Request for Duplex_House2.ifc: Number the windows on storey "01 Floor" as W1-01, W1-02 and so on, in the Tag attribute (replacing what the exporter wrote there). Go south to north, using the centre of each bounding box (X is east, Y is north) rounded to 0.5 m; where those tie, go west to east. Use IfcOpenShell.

First a look at what the model holds.

```python
import ifcopenshell
import ifcopenshell.util.element
import ifcopenshell.util.placement

model = ifcopenshell.open("Duplex_House2.ifc")
print(model.schema)
storey = next(s for s in model.by_type("IfcBuildingStorey") if s.Name == "01 Floor")
windows = [e for e in ifcopenshell.util.element.get_decomposition(storey) if e.is_a("IfcWindow")]
for e in sorted(windows, key=lambda e: e.id()):
    origin = ifcopenshell.util.placement.get_local_placement(e.ObjectPlacement)[:3, 3]
    print(e.id(), e.Tag, e.Name, origin.round(2) + 0.0, sep=" | ")
```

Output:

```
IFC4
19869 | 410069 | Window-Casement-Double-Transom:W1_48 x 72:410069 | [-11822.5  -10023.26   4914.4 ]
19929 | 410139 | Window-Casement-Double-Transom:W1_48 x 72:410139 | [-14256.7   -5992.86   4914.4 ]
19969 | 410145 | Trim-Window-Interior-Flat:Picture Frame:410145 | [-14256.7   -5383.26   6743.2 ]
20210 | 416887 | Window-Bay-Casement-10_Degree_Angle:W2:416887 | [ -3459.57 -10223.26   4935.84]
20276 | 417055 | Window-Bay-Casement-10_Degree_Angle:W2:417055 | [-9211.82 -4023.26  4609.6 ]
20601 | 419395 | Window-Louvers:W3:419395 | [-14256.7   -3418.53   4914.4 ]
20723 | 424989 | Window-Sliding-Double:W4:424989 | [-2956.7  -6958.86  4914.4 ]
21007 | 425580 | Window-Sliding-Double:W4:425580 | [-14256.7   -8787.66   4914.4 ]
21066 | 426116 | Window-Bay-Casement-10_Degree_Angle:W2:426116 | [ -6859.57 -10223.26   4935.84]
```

```python
import ifcopenshell
import ifcopenshell.geom
import ifcopenshell.util.element
import ifcopenshell.util.shape

model = ifcopenshell.open("Duplex_House2.ifc")
settings = ifcopenshell.geom.settings()
settings.set("use-world-coords", True)


def centre(element):
    shape = ifcopenshell.geom.create_shape(settings, element)
    return ifcopenshell.util.shape.get_bbox_centroid(shape.geometry)


storey = next(s for s in model.by_type("IfcBuildingStorey") if s.Name == "01 Floor")
windows = [e for e in ifcopenshell.util.element.get_decomposition(storey) if e.is_a("IfcWindow")]

# Insertion points can sit at a corner or the storey origin, so sort by the geometry (in metres).
centres = {e: centre(e) for e in windows}
windows.sort(key=lambda e: (round(centres[e][1] / 0.5), centres[e][0]))

for i, e in enumerate(windows, start=1):
    number = f"W1-{i:02d}"
    e.Tag = number
    print(e.id(), number)

model.write("Duplex_House2-out.ifc")
```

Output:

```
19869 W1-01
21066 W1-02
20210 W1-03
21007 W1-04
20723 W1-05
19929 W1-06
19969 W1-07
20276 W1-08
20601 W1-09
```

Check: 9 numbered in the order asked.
